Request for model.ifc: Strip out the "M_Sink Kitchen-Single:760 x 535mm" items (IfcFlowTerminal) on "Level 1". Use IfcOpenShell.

First a look at what the model holds.

```python
import ifcopenshell
import ifcopenshell.util.element

model = ifcopenshell.open("model.ifc")
print(model.schema)
storey = next(s for s in model.by_type("IfcBuildingStorey") if s.Name == "Level 1")
terminals = [e for e in ifcopenshell.util.element.get_decomposition(storey) if e.is_a("IfcFlowTerminal")]
seen = {}
for e in terminals:
    element_type = ifcopenshell.util.element.get_type(e)
    name = element_type.Name if element_type not in (None, e) else None
    seen[name] = seen.get(name, 0) + 1
for name, count in sorted(seen.items(), key=str):
    print(count, "x", name)
```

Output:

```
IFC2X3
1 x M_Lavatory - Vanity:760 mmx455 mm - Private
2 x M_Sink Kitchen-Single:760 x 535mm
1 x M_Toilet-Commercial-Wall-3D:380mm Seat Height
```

```python
import ifcopenshell
import ifcopenshell.api.root
import ifcopenshell.util.element

model = ifcopenshell.open("model.ifc")

storey = next(s for s in model.by_type("IfcBuildingStorey") if s.Name == "Level 1")
terminals = [e for e in ifcopenshell.util.element.get_decomposition(storey) if e.is_a("IfcFlowTerminal")]
targets = [e for e in terminals if (t := ifcopenshell.util.element.get_type(e)) not in (None, e) and t.Name == "M_Sink Kitchen-Single:760 x 535mm"]

for e in targets:
    ifcopenshell.api.root.remove_product(model, product=e)
print(len(targets), "removed")

model.write("model-out.ifc")
```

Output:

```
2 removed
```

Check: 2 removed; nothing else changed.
